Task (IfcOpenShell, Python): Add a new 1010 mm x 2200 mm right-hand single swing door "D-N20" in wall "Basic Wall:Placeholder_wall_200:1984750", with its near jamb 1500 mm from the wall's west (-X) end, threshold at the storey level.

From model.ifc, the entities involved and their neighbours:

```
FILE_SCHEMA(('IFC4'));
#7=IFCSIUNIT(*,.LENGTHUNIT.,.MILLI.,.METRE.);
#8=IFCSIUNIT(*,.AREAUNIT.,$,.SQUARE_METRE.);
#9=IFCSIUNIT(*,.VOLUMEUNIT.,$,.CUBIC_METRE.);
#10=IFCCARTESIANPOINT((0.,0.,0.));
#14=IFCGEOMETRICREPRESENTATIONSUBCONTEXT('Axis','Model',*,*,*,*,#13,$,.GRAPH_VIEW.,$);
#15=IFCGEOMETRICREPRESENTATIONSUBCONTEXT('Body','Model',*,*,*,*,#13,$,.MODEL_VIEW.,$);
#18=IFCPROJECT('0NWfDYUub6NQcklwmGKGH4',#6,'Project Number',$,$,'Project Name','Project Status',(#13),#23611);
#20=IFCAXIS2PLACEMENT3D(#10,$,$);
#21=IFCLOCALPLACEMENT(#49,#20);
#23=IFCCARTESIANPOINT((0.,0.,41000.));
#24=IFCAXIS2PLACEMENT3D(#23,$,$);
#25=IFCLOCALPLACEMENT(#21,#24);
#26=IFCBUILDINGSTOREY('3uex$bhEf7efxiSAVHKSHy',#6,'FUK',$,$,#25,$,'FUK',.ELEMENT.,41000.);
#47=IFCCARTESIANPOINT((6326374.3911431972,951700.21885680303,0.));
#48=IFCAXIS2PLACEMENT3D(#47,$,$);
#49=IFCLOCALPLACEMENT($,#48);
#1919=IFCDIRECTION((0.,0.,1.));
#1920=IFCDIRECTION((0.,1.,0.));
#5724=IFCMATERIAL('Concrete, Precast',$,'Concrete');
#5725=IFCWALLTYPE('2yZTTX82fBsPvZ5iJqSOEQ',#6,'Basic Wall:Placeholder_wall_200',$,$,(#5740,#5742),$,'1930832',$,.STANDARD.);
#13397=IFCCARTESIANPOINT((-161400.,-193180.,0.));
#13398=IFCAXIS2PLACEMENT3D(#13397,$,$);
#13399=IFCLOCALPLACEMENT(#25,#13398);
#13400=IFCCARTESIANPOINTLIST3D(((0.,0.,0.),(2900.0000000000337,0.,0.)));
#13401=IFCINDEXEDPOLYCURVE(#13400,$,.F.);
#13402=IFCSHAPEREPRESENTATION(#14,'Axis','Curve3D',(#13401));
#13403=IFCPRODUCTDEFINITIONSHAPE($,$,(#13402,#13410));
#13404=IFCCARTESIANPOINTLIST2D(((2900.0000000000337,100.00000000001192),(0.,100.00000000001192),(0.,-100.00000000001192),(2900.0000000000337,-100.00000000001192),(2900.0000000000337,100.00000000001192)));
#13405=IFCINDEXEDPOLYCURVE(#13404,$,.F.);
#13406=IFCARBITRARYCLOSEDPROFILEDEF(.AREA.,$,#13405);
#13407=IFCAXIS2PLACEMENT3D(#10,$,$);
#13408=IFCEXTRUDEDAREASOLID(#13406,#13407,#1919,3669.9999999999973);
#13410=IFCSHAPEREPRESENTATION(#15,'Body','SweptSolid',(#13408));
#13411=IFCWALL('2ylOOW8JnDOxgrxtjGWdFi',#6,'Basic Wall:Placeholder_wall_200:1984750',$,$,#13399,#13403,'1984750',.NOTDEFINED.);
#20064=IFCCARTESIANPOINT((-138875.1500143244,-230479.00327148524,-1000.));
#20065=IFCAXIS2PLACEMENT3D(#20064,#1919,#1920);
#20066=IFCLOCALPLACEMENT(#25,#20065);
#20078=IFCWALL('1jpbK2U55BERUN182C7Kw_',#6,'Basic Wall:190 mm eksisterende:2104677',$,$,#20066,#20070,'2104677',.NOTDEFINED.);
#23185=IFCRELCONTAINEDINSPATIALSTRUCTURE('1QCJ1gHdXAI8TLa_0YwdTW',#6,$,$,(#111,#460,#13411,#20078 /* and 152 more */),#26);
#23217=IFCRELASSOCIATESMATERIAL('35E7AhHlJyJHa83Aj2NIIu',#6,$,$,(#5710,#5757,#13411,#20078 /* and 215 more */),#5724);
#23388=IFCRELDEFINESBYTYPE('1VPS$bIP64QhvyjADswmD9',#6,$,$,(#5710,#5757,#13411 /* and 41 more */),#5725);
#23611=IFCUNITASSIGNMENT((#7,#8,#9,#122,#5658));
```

```python
import numpy as np
import ifcopenshell
import ifcopenshell.api.feature
import ifcopenshell.api.geometry
import ifcopenshell.api.root
import ifcopenshell.api.spatial
import ifcopenshell.geom
import ifcopenshell.util.element
import ifcopenshell.util.placement
import ifcopenshell.util.representation
import ifcopenshell.util.shape
import ifcopenshell.util.unit

model = ifcopenshell.open("model.ifc")
unit_scale = ifcopenshell.util.unit.calculate_unit_scale(model)
settings = ifcopenshell.geom.settings()


def volume(element):
    """Net volume in cubic metres, openings subtracted."""
    shape = ifcopenshell.geom.create_shape(settings, element)
    return ifcopenshell.util.shape.get_volume(shape.geometry)


wall = model.by_guid("2ylOOW8JnDOxgrxtjGWdFi")
storey = ifcopenshell.util.element.get_container(wall, ifc_class="IfcBuildingStorey")
context = ifcopenshell.util.representation.get_context(model, "Model", "Body", "MODEL_VIEW")
before = volume(wall)

width, height, from_end, sill = 1.01, 2.2, 1.5, 0.0  # metres

# The wall runs along its own X axis, and the end named is its -X end.
wall_shape = ifcopenshell.geom.create_shape(settings, wall)
x, y, z = ifcopenshell.util.shape.get_vertices(wall_shape.geometry).T
start = x.min() + from_end
face, thickness = float(y.min()), float(y.max() - y.min())
wall_matrix = ifcopenshell.util.placement.get_local_placement(wall.ObjectPlacement)
level = ifcopenshell.util.placement.get_local_placement(storey.ObjectPlacement)[2, 3]


def in_wall(x, y):
    """Placement at x, y metres in the wall's axes, at sill height."""
    matrix = wall_matrix.copy()
    matrix[:, 3] = wall_matrix @ np.array([x / unit_scale, y / unit_scale, 0.0, 1.0])
    matrix[2, 3] = level + sill / unit_scale
    return matrix


# Opening: a box that overshoots both wall faces by 50 mm.
opening = ifcopenshell.api.root.create_entity(model, ifc_class="IfcOpeningElement", predefined_type="OPENING")
box = ifcopenshell.api.geometry.add_wall_representation(
    model, context=context, length=width, height=height, thickness=thickness + 0.1
)
ifcopenshell.api.geometry.assign_representation(model, product=opening, representation=box)
ifcopenshell.api.geometry.edit_object_placement(model, product=opening, matrix=in_wall(start, face - 0.05), is_si=False)
ifcopenshell.api.feature.add_feature(model, feature=opening, element=wall)

door = ifcopenshell.api.root.create_entity(model, ifc_class="IfcDoor", name="D-N20", predefined_type="DOOR")
door.OverallWidth, door.OverallHeight = width / unit_scale, height / unit_scale
door.OperationType = "SINGLE_SWING_RIGHT"
body = ifcopenshell.api.geometry.add_door_representation(
    model,
    context=context,
    overall_width=door.OverallWidth,
    overall_height=door.OverallHeight,
    operation_type="SINGLE_SWING_RIGHT",
    lining_properties={"LiningDepth": thickness / unit_scale, "ThresholdDepth": thickness / unit_scale},
)
ifcopenshell.api.geometry.assign_representation(model, product=door, representation=body)
ifcopenshell.api.spatial.assign_container(model, products=[door], relating_structure=storey)
ifcopenshell.api.feature.add_filling(model, opening=opening, element=door)

# The lining spans the wall, so the door starts at the wall face.
ifcopenshell.api.geometry.edit_object_placement(model, product=door, matrix=in_wall(start, face), is_si=False)

after = volume(wall)

print(f"wall volume {before:.3f} -> {after:.3f} m3")

model.write("model_v2.ifc")
```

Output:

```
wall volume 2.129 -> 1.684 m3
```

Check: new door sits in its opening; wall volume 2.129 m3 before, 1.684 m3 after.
